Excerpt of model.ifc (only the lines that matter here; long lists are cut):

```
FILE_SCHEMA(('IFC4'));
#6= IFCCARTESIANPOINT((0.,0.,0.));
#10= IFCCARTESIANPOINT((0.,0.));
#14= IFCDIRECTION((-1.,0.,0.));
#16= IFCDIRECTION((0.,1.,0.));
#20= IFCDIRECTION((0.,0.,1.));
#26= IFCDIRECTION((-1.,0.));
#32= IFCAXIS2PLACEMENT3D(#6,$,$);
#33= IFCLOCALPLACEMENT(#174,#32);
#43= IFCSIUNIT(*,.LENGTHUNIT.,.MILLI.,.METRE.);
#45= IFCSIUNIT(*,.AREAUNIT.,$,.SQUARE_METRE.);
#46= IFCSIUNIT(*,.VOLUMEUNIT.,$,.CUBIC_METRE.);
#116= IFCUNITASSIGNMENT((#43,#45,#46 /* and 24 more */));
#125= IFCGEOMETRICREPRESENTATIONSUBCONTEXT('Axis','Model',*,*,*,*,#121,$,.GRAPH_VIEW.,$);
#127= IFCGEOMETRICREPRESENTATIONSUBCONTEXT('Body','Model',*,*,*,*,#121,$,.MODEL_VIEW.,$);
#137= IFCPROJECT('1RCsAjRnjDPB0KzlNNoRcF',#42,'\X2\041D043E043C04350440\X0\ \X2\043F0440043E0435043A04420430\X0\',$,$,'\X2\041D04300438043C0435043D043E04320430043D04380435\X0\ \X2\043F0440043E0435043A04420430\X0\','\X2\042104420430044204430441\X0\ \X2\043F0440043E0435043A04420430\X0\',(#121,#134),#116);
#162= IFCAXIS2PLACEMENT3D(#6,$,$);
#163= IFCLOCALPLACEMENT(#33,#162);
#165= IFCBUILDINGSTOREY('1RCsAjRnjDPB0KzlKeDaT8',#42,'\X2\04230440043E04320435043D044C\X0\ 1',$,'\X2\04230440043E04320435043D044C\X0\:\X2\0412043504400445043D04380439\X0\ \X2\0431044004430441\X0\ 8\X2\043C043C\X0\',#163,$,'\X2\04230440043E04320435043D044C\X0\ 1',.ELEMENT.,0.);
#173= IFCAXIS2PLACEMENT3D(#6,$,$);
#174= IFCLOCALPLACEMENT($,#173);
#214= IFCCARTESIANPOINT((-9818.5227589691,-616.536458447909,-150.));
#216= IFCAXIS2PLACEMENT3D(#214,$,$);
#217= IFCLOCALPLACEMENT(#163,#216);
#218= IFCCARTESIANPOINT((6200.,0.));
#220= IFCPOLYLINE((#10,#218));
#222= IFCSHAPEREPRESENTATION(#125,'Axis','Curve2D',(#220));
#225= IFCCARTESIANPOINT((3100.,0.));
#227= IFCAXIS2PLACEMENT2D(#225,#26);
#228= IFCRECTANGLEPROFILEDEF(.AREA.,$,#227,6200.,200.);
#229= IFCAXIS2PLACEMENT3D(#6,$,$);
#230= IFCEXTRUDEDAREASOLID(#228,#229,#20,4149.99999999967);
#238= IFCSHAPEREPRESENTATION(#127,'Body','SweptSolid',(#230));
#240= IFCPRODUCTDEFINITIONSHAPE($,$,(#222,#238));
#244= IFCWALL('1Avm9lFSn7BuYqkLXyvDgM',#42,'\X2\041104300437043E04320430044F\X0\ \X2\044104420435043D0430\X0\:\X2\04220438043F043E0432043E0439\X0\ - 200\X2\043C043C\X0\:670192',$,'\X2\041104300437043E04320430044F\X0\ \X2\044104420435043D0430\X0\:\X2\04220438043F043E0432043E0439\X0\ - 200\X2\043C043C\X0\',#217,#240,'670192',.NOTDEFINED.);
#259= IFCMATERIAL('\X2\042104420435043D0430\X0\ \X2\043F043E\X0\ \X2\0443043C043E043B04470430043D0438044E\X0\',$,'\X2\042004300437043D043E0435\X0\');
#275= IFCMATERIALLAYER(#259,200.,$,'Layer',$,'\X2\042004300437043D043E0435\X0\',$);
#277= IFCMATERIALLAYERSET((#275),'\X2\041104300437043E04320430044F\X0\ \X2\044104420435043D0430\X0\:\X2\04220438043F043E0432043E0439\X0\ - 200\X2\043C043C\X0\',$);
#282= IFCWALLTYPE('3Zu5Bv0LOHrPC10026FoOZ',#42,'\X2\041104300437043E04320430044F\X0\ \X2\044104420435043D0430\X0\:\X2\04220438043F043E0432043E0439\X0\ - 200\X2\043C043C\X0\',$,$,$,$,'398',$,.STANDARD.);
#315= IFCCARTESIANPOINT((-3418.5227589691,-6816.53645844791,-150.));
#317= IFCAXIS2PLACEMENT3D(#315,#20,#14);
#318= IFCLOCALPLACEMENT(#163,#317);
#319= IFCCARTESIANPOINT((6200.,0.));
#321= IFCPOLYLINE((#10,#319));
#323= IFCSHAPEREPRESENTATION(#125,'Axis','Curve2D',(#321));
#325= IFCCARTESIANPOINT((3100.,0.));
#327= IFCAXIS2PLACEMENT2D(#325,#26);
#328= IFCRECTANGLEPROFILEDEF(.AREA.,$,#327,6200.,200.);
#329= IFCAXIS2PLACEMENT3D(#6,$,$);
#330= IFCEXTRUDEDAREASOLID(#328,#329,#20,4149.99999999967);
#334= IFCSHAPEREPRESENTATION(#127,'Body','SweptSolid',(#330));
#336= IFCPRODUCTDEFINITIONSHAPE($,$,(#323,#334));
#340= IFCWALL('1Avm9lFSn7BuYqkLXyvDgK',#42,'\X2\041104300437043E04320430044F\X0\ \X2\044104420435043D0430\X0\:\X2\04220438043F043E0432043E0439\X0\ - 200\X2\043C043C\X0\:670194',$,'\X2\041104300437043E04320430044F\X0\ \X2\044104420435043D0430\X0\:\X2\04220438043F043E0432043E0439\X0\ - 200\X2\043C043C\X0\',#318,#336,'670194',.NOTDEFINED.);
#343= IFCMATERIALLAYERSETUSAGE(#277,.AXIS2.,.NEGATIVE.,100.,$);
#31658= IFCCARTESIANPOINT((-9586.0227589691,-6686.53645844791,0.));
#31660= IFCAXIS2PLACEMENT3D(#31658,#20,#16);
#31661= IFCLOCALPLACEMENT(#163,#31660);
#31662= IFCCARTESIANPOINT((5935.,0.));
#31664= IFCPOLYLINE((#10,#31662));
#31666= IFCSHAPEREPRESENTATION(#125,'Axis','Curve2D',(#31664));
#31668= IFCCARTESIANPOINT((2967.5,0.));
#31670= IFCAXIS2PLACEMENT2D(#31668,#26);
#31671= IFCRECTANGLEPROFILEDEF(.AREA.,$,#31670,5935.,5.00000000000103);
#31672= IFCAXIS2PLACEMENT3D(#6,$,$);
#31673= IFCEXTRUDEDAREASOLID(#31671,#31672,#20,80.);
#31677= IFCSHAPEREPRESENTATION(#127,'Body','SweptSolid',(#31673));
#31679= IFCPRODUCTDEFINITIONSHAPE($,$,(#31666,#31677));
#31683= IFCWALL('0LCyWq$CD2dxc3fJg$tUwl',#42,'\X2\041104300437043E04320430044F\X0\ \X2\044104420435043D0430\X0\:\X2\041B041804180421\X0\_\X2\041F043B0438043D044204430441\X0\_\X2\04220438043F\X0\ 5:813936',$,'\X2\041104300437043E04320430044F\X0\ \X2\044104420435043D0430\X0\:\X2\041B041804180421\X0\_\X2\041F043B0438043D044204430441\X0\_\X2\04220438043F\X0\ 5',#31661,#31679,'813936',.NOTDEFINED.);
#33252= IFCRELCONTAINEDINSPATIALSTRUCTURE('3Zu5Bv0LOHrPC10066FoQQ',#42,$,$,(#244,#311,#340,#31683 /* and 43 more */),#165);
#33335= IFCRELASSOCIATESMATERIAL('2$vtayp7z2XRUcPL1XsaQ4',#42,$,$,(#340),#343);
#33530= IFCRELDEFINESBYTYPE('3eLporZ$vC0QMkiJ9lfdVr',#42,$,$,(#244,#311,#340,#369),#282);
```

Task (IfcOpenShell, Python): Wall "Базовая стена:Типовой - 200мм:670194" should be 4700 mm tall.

```python
import ifcopenshell
import ifcopenshell.geom
import ifcopenshell.util.representation
import ifcopenshell.util.shape
import ifcopenshell.util.unit

model = ifcopenshell.open("model.ifc")
unit_scale = ifcopenshell.util.unit.calculate_unit_scale(model)
settings = ifcopenshell.geom.settings()


def volume(element):
    """Net volume in cubic metres, openings subtracted."""
    shape = ifcopenshell.geom.create_shape(settings, element)
    return ifcopenshell.util.shape.get_volume(shape.geometry)


wall = model.by_guid("1Avm9lFSn7BuYqkLXyvDgK")
before = volume(wall)

body = ifcopenshell.util.representation.get_representation(wall, "Model", "Body")
solid = body.Items[0]
old_height = solid.Depth
solid.Depth = 4.7 / unit_scale
after = volume(wall)

print(f"height {old_height:g} -> {solid.Depth:g}, volume {before:.3f} -> {after:.3f} m3")

model.write("model_v2.ifc")
```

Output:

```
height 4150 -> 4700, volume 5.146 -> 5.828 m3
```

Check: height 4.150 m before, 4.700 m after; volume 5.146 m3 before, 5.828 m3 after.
